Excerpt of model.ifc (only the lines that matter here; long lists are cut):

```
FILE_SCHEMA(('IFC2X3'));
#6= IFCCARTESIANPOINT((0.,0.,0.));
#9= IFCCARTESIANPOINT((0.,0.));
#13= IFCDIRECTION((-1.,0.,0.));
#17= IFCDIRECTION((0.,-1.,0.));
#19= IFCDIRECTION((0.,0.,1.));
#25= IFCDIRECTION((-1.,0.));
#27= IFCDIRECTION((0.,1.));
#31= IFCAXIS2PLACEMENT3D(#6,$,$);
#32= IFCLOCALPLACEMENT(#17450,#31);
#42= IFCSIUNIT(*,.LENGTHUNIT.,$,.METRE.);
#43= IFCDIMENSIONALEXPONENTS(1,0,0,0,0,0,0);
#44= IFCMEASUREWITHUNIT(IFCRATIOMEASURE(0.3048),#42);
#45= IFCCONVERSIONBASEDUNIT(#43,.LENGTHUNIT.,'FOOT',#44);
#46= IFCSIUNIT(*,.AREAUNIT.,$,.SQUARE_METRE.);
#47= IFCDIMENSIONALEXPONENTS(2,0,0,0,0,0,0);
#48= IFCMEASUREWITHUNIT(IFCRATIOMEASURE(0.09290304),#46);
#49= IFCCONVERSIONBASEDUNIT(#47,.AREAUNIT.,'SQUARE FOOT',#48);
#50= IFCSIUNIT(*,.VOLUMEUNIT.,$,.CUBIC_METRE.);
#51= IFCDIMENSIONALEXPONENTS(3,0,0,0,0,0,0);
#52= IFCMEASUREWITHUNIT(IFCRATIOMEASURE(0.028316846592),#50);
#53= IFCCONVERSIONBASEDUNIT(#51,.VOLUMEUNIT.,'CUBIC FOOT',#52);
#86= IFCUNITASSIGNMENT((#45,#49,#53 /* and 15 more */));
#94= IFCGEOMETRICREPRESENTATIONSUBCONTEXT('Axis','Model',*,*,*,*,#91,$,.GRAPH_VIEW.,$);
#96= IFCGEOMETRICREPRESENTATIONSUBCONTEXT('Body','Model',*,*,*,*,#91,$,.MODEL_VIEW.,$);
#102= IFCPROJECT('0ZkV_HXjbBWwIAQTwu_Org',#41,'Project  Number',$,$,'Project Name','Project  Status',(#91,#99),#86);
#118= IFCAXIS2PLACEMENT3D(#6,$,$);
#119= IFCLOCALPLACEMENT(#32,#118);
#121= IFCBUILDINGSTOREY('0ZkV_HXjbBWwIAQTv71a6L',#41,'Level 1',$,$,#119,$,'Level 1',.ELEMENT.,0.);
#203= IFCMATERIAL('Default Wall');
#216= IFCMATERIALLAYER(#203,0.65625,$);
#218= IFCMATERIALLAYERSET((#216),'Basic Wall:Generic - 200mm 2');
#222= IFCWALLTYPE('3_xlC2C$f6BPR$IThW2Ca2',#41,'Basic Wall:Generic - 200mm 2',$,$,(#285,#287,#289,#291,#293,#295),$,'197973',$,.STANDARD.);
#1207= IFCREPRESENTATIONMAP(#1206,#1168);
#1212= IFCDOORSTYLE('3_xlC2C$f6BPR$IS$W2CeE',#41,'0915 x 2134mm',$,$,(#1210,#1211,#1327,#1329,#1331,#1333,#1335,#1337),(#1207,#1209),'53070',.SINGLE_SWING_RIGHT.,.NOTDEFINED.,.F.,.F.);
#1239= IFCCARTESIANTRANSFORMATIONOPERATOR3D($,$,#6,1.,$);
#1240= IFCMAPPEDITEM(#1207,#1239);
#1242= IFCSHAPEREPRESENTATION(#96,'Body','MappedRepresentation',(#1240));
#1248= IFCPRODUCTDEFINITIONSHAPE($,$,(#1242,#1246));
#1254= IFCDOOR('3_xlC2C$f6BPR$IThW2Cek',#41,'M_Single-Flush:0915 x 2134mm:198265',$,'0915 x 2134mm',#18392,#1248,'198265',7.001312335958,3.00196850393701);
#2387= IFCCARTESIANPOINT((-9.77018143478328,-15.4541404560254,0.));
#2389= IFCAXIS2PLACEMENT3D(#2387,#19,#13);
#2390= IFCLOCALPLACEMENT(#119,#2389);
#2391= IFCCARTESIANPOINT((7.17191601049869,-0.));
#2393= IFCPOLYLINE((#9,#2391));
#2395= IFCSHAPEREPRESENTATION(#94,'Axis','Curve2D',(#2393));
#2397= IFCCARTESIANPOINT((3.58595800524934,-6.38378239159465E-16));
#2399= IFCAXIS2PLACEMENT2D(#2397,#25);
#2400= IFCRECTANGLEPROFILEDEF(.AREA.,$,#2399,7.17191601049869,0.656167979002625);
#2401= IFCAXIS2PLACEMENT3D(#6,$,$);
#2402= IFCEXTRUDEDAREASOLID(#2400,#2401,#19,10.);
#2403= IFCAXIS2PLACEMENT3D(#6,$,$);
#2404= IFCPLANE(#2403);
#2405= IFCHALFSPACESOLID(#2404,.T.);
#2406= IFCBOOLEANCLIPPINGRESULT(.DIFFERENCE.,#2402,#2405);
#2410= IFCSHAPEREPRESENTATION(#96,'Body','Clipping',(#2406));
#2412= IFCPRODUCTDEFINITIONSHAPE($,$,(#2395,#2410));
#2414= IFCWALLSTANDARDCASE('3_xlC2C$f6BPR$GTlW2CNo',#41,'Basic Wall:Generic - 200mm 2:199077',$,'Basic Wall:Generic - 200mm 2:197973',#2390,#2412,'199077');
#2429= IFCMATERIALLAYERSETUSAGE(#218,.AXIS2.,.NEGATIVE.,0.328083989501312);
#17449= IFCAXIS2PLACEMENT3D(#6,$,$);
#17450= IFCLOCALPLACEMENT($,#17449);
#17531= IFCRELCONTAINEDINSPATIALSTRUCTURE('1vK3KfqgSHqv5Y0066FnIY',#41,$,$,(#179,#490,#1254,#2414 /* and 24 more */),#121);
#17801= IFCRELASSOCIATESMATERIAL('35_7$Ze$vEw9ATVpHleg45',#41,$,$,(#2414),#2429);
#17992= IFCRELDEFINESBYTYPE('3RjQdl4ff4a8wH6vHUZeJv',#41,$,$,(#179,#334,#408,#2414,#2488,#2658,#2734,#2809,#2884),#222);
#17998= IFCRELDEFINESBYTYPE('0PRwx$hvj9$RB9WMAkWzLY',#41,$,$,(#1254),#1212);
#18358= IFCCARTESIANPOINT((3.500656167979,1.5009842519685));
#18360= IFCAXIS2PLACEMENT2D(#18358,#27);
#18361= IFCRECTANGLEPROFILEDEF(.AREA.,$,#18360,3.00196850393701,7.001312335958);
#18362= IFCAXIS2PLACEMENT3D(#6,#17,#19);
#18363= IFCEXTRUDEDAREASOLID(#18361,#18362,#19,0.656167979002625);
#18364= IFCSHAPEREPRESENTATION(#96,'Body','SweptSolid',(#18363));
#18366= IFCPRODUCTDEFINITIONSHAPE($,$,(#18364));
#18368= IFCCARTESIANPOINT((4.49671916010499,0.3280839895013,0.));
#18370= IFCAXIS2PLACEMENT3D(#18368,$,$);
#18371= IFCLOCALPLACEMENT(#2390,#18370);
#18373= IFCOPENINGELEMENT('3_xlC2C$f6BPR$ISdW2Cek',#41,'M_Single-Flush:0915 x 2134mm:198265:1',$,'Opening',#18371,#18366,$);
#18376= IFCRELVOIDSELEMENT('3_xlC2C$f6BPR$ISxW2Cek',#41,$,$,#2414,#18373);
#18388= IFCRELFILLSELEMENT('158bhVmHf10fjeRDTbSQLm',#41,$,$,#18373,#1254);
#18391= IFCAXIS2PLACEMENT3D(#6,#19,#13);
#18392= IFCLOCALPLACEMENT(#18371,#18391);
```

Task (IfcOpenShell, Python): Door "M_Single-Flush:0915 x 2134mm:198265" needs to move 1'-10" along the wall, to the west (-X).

```python
import ifcopenshell
import ifcopenshell.api.geometry
import ifcopenshell.util.placement
import ifcopenshell.util.unit

model = ifcopenshell.open("model.ifc")
unit_scale = ifcopenshell.util.unit.calculate_unit_scale(model)

door = model.by_guid("3_xlC2C$f6BPR$IThW2Cek")
opening = door.FillsVoids[0].RelatingOpeningElement
wall = opening.VoidsElements[0].RelatingBuildingElement

wall_matrix = ifcopenshell.util.placement.get_local_placement(wall.ObjectPlacement)
shift = wall_matrix[:3, 0] * 22 * 0.0254 / unit_scale
before = ifcopenshell.util.placement.get_local_placement(door.ObjectPlacement)[:3, 3].copy()

# The door is placed relative to its opening, so it follows when the opening moves.
matrix = ifcopenshell.util.placement.get_local_placement(opening.ObjectPlacement)
matrix[:3, 3] += shift
ifcopenshell.api.geometry.edit_object_placement(
    model, product=opening, matrix=matrix, is_si=False, should_transform_children=True
)

after = ifcopenshell.util.placement.get_local_placement(door.ObjectPlacement)[:3, 3]
print("door moved by", (after - before).round(3) + 0.0)

model.write("model_updated.ifc")
```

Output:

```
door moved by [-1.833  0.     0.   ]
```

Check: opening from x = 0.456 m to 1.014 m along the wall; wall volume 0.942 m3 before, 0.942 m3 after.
